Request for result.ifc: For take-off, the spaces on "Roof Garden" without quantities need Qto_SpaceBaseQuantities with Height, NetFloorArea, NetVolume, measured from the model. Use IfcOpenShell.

First a look at what the model holds.

```python
import ifcopenshell
import ifcopenshell.util.element
import ifcopenshell.util.unit

model = ifcopenshell.open("result.ifc")
print(model.schema)
for unit_type in ("LENGTHUNIT", "AREAUNIT", "VOLUMEUNIT"):
    print(unit_type, ifcopenshell.util.unit.calculate_unit_scale(model, unit_type))
storey = next(s for s in model.by_type("IfcBuildingStorey") if s.Name == "Roof Garden")
spaces = [e for e in ifcopenshell.util.element.get_decomposition(storey) if e.is_a("IfcSpace")]
for e in sorted(spaces, key=lambda e: e.id()):
    print(e.id(), e.is_a(), e.Name, list(ifcopenshell.util.element.get_psets(e, qtos_only=True)), sep=" | ")
```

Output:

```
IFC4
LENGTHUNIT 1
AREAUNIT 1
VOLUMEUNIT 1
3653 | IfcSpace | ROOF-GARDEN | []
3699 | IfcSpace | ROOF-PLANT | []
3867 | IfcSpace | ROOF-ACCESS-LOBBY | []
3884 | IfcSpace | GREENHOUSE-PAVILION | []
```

```python
import ifcopenshell
import ifcopenshell.api.pset
import ifcopenshell.geom
import ifcopenshell.util.element
import ifcopenshell.util.shape
import ifcopenshell.util.unit

model = ifcopenshell.open("result.ifc")
unit_scale = ifcopenshell.util.unit.calculate_unit_scale(model)
area_scale = ifcopenshell.util.unit.calculate_unit_scale(model, "AREAUNIT")
volume_scale = ifcopenshell.util.unit.calculate_unit_scale(model, "VOLUMEUNIT")
settings = ifcopenshell.geom.settings()

storey = next(s for s in model.by_type("IfcBuildingStorey") if s.Name == "Roof Garden")
spaces = [e for e in ifcopenshell.util.element.get_decomposition(storey) if e.is_a("IfcSpace")]

for e in sorted(spaces, key=lambda e: e.id()):
    if ifcopenshell.util.element.get_psets(e, qtos_only=True, should_inherit=False):
        continue
    # Geometry comes back in metres, in the element's own axes.
    shape = ifcopenshell.geom.create_shape(settings, e)
    values = {
        "Height": ifcopenshell.util.shape.get_z(shape.geometry) / unit_scale,
        "NetFloorArea": ifcopenshell.util.shape.get_footprint_area(shape.geometry) / area_scale,
        "NetVolume": ifcopenshell.util.shape.get_volume(shape.geometry) / volume_scale,
    }
    qto = ifcopenshell.api.pset.add_qto(model, product=e, name="Qto_SpaceBaseQuantities")
    ifcopenshell.api.pset.edit_qto(model, qto=qto, properties=values)
    print(e.id(), {k: round(v, 3) for k, v in values.items()})

model.write("result_rev.ifc")
```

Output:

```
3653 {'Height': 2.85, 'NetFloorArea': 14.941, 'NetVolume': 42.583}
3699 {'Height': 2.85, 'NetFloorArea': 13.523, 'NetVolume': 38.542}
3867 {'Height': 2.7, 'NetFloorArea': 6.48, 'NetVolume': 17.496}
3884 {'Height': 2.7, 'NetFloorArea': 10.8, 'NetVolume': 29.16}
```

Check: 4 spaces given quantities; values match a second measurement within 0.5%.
